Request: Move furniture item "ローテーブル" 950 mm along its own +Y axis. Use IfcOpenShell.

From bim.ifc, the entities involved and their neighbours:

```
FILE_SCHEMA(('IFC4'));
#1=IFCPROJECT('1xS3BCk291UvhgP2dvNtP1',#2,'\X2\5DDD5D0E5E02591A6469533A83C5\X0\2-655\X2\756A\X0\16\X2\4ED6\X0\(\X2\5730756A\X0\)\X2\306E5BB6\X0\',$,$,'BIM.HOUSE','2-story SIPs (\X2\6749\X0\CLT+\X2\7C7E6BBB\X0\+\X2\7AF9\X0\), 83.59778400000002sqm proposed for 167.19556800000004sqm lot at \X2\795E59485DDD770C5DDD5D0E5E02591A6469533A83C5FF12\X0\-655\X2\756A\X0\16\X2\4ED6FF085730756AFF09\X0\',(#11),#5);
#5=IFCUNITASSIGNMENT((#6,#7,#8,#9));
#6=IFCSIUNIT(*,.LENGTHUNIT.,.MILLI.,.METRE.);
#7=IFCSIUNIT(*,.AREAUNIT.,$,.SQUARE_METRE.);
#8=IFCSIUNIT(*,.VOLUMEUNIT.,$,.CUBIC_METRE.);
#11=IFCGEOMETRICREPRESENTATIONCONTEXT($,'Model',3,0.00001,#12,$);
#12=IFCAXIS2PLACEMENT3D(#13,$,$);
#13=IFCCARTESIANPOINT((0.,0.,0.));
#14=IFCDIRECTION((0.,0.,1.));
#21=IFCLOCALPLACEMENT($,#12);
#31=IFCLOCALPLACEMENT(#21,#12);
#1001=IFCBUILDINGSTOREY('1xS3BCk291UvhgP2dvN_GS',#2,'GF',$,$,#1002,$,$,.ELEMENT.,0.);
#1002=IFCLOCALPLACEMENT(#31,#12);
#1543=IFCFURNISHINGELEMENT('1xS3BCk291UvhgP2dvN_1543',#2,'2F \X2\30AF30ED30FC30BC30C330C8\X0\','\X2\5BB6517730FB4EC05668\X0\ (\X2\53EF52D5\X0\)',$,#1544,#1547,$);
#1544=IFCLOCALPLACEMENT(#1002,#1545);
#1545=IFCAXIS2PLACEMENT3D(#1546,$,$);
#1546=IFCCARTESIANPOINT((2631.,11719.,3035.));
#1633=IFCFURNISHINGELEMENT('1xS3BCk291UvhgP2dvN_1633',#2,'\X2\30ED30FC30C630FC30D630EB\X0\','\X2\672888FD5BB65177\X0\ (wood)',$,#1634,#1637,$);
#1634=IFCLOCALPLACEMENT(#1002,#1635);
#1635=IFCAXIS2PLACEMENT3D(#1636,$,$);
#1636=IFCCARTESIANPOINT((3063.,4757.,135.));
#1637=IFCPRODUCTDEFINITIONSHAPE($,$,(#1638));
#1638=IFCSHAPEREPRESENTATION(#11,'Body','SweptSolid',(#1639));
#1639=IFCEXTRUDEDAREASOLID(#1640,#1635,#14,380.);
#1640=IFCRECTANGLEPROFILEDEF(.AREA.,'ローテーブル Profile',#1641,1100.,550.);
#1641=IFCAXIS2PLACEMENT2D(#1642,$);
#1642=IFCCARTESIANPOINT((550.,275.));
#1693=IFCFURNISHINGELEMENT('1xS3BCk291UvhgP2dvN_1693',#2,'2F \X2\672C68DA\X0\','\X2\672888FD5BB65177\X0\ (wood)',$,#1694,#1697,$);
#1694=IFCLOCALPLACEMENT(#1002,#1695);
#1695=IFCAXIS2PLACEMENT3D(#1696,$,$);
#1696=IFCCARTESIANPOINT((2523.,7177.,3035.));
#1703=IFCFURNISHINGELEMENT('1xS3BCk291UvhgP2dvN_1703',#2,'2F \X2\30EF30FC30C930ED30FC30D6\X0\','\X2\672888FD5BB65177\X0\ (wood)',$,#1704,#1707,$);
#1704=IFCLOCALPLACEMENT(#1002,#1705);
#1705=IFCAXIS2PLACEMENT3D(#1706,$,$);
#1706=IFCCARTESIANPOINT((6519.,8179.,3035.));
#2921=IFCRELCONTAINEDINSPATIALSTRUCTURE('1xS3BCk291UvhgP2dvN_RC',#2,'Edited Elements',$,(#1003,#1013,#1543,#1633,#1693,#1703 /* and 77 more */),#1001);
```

```python
import ifcopenshell
import ifcopenshell.api.geometry
import ifcopenshell.util.placement

model = ifcopenshell.open("bim.ifc")

item = model.by_guid("1xS3BCk291UvhgP2dvN_1633")
matrix = ifcopenshell.util.placement.get_local_placement(item.ObjectPlacement)
matrix[:3, 3] += matrix[:3, 1] * 950.0
ifcopenshell.api.geometry.edit_object_placement(model, product=item, matrix=matrix, is_si=False)

print(ifcopenshell.util.placement.get_local_placement(item.ObjectPlacement).round(3) + 0.0)

model.write("bim-out.ifc")
```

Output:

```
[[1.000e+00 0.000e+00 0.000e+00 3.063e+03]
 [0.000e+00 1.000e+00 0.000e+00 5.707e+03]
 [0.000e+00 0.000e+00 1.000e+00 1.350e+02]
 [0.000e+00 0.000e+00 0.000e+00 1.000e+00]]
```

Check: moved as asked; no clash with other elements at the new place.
